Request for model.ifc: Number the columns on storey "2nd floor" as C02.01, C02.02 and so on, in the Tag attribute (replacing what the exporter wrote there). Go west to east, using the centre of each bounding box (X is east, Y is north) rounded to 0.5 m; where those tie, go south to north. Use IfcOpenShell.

First a look at what the model holds.

```python
import ifcopenshell
import ifcopenshell.util.element
import ifcopenshell.util.placement

model = ifcopenshell.open("model.ifc")
print(model.schema)
storey = next(s for s in model.by_type("IfcBuildingStorey") if s.Name == "2nd floor")
columns = [e for e in ifcopenshell.util.element.get_decomposition(storey) if e.is_a("IfcColumn")]
for e in sorted(columns, key=lambda e: e.id()):
    origin = ifcopenshell.util.placement.get_local_placement(e.ObjectPlacement)[:3, 3]
    print(e.id(), e.Tag, e.Name, origin.round(2) + 0.0, sep=" | ")
```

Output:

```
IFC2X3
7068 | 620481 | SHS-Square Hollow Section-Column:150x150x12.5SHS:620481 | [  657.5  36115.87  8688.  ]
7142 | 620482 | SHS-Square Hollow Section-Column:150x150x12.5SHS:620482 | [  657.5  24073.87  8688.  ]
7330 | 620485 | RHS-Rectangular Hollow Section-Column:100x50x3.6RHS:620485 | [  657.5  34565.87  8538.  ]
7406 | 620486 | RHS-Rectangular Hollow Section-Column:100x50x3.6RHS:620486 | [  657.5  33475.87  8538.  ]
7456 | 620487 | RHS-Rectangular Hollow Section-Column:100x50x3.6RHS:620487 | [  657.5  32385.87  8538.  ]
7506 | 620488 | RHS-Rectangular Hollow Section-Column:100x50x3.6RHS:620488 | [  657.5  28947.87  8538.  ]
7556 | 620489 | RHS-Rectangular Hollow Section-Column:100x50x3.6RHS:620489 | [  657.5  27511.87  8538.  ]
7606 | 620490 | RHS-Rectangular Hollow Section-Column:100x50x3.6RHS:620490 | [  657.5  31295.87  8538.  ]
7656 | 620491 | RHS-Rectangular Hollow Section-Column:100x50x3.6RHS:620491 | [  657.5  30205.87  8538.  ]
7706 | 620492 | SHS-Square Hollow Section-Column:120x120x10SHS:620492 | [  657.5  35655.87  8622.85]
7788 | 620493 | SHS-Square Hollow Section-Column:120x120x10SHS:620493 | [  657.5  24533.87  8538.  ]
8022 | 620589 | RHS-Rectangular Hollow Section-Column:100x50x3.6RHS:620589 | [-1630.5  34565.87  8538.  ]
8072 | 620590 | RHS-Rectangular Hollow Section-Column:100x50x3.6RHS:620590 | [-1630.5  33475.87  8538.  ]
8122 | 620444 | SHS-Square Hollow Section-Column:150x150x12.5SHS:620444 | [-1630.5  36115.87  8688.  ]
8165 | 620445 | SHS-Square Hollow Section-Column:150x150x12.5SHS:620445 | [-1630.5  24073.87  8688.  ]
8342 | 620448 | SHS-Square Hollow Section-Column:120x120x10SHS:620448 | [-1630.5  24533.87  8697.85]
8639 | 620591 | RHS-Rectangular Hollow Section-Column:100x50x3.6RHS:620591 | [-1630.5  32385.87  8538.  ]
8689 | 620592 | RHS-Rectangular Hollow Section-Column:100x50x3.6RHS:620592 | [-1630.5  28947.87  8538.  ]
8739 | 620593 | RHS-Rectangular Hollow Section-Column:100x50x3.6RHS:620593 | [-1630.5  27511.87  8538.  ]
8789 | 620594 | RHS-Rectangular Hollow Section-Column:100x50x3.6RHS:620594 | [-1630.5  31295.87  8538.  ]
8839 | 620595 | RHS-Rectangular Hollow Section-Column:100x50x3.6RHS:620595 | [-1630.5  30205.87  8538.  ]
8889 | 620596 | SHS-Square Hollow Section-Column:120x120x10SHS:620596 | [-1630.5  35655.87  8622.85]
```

```python
import ifcopenshell
import ifcopenshell.geom
import ifcopenshell.util.element
import ifcopenshell.util.shape

model = ifcopenshell.open("model.ifc")
settings = ifcopenshell.geom.settings()
settings.set("use-world-coords", True)


def centre(element):
    shape = ifcopenshell.geom.create_shape(settings, element)
    return ifcopenshell.util.shape.get_bbox_centroid(shape.geometry)


storey = next(s for s in model.by_type("IfcBuildingStorey") if s.Name == "2nd floor")
columns = [e for e in ifcopenshell.util.element.get_decomposition(storey) if e.is_a("IfcColumn")]

# Insertion points can sit at a corner or the storey origin, so sort by the geometry (in metres).
centres = {e: centre(e) for e in columns}
columns.sort(key=lambda e: (round(centres[e][0] / 0.5), centres[e][1]))

for i, e in enumerate(columns, start=1):
    number = f"C02.{i:02d}"
    e.Tag = number
    print(e.id(), number)

model.write("model_updated.ifc")
```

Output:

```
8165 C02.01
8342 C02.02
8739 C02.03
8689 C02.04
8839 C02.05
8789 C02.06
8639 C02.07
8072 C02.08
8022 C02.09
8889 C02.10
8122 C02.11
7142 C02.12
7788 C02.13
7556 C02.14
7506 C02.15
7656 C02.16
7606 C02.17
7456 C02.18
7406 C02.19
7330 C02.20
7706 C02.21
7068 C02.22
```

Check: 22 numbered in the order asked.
